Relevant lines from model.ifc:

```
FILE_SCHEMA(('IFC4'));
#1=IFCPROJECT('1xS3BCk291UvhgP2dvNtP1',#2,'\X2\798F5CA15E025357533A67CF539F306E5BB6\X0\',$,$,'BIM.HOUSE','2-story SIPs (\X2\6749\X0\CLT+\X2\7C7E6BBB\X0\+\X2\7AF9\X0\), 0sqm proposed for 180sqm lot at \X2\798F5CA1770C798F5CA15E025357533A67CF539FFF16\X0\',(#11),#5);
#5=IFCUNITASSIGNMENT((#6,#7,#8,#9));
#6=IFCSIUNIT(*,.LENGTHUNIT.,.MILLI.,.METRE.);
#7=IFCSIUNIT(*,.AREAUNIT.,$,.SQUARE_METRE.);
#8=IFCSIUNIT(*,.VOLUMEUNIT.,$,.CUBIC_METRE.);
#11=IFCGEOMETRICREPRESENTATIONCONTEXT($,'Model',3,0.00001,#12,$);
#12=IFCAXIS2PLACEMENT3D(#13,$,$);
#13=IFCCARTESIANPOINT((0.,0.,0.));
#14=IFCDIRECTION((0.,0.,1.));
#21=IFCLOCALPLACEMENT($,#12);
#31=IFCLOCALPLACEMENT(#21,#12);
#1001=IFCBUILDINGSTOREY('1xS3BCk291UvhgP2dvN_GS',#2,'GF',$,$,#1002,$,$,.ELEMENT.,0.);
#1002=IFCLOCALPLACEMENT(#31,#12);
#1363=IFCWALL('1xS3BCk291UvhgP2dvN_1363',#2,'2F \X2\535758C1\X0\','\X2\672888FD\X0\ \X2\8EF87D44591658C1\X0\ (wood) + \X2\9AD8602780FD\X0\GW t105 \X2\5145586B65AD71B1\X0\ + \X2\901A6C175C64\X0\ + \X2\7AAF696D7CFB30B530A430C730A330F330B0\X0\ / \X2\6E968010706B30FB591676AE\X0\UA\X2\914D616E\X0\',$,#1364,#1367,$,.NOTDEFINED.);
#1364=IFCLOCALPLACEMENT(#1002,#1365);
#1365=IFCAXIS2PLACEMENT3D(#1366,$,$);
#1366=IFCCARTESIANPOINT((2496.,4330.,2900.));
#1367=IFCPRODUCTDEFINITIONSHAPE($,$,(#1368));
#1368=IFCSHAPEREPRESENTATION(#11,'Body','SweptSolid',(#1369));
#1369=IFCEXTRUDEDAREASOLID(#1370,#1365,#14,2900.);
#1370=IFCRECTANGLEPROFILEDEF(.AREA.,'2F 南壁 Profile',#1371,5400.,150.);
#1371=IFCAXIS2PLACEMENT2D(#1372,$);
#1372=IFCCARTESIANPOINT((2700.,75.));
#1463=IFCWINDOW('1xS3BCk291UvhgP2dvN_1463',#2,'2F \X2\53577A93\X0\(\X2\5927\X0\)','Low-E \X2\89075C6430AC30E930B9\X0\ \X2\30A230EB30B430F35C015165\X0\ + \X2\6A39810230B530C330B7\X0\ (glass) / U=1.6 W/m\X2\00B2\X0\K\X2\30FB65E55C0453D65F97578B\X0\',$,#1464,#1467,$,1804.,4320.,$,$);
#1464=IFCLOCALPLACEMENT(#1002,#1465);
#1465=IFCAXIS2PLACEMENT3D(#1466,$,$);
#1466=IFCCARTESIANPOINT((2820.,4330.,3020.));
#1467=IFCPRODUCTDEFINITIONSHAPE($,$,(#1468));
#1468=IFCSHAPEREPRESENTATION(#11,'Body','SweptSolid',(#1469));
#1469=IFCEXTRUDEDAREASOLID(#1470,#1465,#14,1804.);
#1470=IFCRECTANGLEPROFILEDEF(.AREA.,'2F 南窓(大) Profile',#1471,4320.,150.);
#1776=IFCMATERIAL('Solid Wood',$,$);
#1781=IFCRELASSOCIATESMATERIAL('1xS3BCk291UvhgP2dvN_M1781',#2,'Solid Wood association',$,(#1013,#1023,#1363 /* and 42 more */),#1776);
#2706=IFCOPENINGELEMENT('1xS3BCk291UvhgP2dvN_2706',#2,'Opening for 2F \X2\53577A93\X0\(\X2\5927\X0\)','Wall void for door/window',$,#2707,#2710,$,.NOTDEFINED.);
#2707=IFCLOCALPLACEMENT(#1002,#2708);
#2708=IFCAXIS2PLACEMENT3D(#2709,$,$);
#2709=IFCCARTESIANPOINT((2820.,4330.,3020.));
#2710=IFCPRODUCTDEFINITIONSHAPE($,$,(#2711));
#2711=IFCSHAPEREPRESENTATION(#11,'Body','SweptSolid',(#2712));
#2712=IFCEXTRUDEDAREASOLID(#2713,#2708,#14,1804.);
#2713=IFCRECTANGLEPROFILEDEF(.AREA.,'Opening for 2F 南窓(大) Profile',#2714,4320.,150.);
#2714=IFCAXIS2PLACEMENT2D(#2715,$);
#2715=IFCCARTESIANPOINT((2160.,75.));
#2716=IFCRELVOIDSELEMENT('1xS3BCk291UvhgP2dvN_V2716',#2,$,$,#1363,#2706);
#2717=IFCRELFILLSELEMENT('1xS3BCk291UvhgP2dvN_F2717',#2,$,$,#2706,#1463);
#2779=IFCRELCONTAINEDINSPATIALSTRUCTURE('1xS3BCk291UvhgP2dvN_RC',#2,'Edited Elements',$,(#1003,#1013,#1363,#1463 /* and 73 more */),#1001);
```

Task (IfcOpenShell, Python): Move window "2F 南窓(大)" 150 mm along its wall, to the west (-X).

```python
import ifcopenshell
import ifcopenshell.api.geometry
import ifcopenshell.util.placement
import ifcopenshell.util.unit

model = ifcopenshell.open("model.ifc")
unit_scale = ifcopenshell.util.unit.calculate_unit_scale(model)

window = model.by_id(1463)
opening = window.FillsVoids[0].RelatingOpeningElement
wall = opening.VoidsElements[0].RelatingBuildingElement

wall_matrix = ifcopenshell.util.placement.get_local_placement(wall.ObjectPlacement)
shift = wall_matrix[:3, 0] * -0.15 / unit_scale
before = ifcopenshell.util.placement.get_local_placement(window.ObjectPlacement)[:3, 3].copy()

# The window is not placed relative to its opening, so move both.
for product in (opening, window):
    matrix = ifcopenshell.util.placement.get_local_placement(product.ObjectPlacement)
    matrix[:3, 3] += shift
    ifcopenshell.api.geometry.edit_object_placement(model, product=product, matrix=matrix, is_si=False)

after = ifcopenshell.util.placement.get_local_placement(window.ObjectPlacement)[:3, 3]
print("window moved by", (after - before).round(3) + 0.0)

model.write("model_rev.ifc")
```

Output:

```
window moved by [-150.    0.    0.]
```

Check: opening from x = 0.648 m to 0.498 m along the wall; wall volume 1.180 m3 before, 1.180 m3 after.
